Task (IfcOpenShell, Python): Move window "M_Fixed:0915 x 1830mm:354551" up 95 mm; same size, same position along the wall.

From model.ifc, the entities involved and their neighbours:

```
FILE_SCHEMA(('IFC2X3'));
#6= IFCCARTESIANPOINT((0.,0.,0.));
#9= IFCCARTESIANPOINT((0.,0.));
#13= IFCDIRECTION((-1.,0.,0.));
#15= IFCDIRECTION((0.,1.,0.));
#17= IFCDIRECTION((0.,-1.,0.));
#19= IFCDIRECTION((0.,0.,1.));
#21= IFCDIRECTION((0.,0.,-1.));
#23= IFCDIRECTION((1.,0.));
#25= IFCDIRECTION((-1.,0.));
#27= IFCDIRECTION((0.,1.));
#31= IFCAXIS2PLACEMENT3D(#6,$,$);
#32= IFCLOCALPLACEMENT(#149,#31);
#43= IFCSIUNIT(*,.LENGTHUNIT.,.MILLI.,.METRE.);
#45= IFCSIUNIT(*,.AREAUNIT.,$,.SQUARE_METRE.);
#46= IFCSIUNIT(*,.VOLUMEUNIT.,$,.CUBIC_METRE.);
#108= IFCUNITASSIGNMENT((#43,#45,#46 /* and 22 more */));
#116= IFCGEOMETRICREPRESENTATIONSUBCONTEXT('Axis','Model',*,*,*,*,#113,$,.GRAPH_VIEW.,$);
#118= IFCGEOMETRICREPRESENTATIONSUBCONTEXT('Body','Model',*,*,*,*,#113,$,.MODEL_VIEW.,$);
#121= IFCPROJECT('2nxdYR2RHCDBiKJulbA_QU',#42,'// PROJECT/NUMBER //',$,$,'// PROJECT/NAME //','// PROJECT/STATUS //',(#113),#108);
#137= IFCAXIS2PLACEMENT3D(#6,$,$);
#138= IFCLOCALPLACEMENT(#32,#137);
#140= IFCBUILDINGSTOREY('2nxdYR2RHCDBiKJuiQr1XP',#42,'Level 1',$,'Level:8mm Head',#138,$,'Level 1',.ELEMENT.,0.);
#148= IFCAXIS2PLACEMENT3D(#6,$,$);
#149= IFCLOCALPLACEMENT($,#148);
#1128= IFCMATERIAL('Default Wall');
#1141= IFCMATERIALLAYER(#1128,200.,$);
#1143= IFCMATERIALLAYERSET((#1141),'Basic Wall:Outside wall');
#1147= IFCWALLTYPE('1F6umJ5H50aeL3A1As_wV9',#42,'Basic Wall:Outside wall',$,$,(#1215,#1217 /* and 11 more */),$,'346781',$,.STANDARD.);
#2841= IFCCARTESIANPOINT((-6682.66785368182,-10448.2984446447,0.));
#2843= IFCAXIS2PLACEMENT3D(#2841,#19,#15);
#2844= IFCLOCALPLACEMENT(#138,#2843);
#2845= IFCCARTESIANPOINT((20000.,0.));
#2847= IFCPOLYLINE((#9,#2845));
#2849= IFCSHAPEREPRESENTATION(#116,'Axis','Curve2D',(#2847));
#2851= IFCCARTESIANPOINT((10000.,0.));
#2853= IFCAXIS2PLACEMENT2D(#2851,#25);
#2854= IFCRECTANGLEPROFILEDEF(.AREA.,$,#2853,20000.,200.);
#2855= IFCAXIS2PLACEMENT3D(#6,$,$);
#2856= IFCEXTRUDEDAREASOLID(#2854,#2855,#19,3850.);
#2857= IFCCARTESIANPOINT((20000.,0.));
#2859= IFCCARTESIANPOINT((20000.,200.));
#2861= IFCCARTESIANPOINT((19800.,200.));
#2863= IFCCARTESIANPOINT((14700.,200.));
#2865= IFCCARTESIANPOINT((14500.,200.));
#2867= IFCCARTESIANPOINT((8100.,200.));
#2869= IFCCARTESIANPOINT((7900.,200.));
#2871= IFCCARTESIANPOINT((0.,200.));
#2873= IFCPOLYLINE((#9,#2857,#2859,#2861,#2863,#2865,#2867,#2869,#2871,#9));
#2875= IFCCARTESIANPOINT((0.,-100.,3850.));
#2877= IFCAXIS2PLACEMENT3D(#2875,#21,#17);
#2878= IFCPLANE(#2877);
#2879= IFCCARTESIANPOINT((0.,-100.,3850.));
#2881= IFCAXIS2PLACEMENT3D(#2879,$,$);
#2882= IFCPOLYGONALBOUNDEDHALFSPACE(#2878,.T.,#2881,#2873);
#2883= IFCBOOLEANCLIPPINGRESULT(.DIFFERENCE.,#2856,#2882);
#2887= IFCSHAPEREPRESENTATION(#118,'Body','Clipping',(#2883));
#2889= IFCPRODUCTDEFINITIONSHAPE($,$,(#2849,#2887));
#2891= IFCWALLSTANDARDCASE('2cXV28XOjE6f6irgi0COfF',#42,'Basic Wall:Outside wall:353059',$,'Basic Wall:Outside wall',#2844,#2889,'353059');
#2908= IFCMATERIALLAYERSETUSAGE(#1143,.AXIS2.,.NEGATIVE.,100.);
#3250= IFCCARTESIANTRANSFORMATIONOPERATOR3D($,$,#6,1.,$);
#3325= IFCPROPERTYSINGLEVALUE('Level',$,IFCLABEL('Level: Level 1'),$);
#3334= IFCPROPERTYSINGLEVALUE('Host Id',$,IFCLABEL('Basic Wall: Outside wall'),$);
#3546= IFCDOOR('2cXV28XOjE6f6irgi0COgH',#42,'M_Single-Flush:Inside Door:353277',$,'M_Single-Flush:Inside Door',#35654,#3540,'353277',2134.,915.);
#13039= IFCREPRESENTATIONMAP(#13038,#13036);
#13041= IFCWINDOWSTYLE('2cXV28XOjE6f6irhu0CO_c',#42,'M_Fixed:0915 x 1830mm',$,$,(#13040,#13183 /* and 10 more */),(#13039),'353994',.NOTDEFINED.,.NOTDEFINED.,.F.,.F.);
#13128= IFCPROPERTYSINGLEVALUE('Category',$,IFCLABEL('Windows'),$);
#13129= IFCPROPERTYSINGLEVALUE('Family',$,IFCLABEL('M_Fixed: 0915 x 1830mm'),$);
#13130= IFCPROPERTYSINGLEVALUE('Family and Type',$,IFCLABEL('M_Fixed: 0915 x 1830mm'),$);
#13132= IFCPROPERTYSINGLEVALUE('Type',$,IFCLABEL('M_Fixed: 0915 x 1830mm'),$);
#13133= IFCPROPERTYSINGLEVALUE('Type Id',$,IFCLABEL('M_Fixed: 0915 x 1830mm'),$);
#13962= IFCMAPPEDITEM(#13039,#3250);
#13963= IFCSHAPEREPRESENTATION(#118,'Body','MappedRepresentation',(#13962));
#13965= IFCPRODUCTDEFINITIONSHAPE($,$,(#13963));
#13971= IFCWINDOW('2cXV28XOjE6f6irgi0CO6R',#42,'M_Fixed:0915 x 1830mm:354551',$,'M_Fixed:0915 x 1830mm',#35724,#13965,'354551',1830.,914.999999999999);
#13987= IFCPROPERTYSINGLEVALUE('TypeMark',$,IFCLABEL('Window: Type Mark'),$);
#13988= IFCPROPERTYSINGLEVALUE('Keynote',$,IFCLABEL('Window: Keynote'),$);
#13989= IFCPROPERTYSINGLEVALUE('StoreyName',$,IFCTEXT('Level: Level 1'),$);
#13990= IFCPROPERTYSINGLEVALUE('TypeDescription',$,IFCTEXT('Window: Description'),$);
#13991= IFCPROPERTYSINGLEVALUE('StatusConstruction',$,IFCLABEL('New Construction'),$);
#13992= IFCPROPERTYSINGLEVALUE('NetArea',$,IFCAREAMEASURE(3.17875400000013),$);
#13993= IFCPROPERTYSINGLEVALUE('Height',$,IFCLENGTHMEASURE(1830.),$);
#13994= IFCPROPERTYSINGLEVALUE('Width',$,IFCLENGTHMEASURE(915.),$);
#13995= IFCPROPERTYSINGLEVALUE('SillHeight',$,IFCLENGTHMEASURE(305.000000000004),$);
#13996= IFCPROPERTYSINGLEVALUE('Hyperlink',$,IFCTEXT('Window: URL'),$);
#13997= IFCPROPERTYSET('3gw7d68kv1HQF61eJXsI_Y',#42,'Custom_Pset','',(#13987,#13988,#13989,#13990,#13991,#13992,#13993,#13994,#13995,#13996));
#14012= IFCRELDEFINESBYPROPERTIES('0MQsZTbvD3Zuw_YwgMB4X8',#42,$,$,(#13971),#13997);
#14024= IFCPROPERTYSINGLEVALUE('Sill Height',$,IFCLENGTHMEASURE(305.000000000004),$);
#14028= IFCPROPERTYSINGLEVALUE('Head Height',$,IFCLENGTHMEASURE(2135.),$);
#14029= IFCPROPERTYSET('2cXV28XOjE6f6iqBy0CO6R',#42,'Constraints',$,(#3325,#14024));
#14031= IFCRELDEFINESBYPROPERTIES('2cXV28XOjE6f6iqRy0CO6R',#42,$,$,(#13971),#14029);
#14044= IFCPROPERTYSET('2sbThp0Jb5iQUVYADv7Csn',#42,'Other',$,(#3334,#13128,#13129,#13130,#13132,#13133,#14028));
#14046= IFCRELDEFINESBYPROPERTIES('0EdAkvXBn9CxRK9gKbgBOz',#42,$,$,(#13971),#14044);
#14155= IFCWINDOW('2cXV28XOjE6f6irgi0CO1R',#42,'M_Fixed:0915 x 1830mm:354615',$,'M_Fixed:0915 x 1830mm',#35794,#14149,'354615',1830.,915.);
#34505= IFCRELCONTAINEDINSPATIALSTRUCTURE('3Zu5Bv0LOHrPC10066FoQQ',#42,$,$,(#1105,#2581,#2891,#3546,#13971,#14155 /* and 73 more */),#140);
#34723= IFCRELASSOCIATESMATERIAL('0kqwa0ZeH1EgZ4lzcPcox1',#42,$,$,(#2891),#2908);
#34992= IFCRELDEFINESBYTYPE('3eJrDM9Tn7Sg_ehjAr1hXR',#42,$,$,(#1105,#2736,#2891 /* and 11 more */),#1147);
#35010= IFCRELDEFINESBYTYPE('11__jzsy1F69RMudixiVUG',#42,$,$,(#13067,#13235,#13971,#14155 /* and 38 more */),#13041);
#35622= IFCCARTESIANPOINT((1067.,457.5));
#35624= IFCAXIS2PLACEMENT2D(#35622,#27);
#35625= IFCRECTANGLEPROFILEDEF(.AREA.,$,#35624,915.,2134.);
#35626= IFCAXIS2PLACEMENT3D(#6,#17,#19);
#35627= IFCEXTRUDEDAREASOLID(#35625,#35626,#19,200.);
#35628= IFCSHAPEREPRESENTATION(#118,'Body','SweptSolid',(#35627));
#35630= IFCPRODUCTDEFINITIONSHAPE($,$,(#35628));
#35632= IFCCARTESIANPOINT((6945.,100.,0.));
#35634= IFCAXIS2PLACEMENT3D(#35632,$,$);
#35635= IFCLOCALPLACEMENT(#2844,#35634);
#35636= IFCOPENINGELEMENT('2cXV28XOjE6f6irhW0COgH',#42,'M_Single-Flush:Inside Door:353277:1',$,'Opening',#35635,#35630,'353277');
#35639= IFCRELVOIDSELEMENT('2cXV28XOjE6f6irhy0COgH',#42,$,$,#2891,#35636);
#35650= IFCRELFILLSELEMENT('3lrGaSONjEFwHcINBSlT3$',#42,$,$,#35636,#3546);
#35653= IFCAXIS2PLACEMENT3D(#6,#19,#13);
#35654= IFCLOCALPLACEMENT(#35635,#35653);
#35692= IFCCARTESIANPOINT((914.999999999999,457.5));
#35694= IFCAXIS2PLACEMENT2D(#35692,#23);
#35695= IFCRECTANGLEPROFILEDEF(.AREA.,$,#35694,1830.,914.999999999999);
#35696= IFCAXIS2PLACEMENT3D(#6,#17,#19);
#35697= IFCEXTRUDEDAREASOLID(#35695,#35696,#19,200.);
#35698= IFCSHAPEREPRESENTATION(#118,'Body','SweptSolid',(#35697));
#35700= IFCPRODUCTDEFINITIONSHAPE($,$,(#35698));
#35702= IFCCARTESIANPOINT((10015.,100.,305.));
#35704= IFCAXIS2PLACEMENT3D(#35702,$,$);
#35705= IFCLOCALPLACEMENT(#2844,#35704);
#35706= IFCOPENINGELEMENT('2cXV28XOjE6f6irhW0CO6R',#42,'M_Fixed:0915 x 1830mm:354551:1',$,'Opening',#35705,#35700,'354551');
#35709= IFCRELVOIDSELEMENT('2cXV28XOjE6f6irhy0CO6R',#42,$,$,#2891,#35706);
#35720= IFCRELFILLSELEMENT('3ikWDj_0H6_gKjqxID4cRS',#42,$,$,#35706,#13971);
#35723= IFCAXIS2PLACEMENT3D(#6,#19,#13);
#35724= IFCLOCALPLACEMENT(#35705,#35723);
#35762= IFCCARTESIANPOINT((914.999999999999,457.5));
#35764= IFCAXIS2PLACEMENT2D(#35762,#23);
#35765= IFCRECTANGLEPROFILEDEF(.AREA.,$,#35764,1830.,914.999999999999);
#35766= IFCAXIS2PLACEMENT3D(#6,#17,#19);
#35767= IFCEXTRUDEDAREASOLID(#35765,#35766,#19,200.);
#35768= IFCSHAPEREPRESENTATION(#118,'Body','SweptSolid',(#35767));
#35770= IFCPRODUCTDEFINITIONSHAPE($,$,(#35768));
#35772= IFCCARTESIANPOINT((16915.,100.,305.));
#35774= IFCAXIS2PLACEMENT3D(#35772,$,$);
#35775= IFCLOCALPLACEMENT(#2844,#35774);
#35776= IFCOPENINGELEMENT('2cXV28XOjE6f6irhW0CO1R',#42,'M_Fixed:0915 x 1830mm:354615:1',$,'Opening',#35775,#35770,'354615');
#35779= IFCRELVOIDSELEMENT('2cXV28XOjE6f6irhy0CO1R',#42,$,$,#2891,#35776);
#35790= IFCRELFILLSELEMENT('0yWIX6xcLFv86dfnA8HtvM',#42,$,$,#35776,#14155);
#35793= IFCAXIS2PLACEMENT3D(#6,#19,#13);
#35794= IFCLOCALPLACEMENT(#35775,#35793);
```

```python
import numpy as np
import ifcopenshell
import ifcopenshell.api.geometry
import ifcopenshell.api.pset
import ifcopenshell.util.element
import ifcopenshell.util.placement
import ifcopenshell.util.unit

model = ifcopenshell.open("model.ifc")
unit_scale = ifcopenshell.util.unit.calculate_unit_scale(model)

window = model.by_guid("2cXV28XOjE6f6irgi0CO6R")
opening = window.FillsVoids[0].RelatingOpeningElement
dz = 95.0

shift = np.array([0.0, 0.0, dz])
# The window is placed relative to its opening, so it follows when the opening moves.
matrix = ifcopenshell.util.placement.get_local_placement(opening.ObjectPlacement)
matrix[:3, 3] += shift
ifcopenshell.api.geometry.edit_object_placement(
    model, product=opening, matrix=matrix, is_si=False, should_transform_children=True
)

# Keep the stored heights in step.
pset = model.by_id(ifcopenshell.util.element.get_pset(window, "Custom_Pset", should_inherit=False)["id"])
ifcopenshell.api.pset.edit_pset(model, pset=pset, properties={
    "SillHeight": model.create_entity("IfcLengthMeasure", ifcopenshell.util.element.get_pset(window, "Constraints", "Sill Height") + dz),
})
pset = model.by_id(ifcopenshell.util.element.get_pset(window, "Constraints", should_inherit=False)["id"])
ifcopenshell.api.pset.edit_pset(model, pset=pset, properties={
    "Sill Height": model.create_entity("IfcLengthMeasure", ifcopenshell.util.element.get_pset(window, "Constraints", "Sill Height") + dz),
})
pset = model.by_id(ifcopenshell.util.element.get_pset(window, "Other", should_inherit=False)["id"])
ifcopenshell.api.pset.edit_pset(model, pset=pset, properties={
    "Head Height": model.create_entity("IfcLengthMeasure", ifcopenshell.util.element.get_pset(window, "Other", "Head Height") + dz),
})

print(f"moved by {dz * unit_scale:+.3f} m")

model.write("model-out.ifc")
```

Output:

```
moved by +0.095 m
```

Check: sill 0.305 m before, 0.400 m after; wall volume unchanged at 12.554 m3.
